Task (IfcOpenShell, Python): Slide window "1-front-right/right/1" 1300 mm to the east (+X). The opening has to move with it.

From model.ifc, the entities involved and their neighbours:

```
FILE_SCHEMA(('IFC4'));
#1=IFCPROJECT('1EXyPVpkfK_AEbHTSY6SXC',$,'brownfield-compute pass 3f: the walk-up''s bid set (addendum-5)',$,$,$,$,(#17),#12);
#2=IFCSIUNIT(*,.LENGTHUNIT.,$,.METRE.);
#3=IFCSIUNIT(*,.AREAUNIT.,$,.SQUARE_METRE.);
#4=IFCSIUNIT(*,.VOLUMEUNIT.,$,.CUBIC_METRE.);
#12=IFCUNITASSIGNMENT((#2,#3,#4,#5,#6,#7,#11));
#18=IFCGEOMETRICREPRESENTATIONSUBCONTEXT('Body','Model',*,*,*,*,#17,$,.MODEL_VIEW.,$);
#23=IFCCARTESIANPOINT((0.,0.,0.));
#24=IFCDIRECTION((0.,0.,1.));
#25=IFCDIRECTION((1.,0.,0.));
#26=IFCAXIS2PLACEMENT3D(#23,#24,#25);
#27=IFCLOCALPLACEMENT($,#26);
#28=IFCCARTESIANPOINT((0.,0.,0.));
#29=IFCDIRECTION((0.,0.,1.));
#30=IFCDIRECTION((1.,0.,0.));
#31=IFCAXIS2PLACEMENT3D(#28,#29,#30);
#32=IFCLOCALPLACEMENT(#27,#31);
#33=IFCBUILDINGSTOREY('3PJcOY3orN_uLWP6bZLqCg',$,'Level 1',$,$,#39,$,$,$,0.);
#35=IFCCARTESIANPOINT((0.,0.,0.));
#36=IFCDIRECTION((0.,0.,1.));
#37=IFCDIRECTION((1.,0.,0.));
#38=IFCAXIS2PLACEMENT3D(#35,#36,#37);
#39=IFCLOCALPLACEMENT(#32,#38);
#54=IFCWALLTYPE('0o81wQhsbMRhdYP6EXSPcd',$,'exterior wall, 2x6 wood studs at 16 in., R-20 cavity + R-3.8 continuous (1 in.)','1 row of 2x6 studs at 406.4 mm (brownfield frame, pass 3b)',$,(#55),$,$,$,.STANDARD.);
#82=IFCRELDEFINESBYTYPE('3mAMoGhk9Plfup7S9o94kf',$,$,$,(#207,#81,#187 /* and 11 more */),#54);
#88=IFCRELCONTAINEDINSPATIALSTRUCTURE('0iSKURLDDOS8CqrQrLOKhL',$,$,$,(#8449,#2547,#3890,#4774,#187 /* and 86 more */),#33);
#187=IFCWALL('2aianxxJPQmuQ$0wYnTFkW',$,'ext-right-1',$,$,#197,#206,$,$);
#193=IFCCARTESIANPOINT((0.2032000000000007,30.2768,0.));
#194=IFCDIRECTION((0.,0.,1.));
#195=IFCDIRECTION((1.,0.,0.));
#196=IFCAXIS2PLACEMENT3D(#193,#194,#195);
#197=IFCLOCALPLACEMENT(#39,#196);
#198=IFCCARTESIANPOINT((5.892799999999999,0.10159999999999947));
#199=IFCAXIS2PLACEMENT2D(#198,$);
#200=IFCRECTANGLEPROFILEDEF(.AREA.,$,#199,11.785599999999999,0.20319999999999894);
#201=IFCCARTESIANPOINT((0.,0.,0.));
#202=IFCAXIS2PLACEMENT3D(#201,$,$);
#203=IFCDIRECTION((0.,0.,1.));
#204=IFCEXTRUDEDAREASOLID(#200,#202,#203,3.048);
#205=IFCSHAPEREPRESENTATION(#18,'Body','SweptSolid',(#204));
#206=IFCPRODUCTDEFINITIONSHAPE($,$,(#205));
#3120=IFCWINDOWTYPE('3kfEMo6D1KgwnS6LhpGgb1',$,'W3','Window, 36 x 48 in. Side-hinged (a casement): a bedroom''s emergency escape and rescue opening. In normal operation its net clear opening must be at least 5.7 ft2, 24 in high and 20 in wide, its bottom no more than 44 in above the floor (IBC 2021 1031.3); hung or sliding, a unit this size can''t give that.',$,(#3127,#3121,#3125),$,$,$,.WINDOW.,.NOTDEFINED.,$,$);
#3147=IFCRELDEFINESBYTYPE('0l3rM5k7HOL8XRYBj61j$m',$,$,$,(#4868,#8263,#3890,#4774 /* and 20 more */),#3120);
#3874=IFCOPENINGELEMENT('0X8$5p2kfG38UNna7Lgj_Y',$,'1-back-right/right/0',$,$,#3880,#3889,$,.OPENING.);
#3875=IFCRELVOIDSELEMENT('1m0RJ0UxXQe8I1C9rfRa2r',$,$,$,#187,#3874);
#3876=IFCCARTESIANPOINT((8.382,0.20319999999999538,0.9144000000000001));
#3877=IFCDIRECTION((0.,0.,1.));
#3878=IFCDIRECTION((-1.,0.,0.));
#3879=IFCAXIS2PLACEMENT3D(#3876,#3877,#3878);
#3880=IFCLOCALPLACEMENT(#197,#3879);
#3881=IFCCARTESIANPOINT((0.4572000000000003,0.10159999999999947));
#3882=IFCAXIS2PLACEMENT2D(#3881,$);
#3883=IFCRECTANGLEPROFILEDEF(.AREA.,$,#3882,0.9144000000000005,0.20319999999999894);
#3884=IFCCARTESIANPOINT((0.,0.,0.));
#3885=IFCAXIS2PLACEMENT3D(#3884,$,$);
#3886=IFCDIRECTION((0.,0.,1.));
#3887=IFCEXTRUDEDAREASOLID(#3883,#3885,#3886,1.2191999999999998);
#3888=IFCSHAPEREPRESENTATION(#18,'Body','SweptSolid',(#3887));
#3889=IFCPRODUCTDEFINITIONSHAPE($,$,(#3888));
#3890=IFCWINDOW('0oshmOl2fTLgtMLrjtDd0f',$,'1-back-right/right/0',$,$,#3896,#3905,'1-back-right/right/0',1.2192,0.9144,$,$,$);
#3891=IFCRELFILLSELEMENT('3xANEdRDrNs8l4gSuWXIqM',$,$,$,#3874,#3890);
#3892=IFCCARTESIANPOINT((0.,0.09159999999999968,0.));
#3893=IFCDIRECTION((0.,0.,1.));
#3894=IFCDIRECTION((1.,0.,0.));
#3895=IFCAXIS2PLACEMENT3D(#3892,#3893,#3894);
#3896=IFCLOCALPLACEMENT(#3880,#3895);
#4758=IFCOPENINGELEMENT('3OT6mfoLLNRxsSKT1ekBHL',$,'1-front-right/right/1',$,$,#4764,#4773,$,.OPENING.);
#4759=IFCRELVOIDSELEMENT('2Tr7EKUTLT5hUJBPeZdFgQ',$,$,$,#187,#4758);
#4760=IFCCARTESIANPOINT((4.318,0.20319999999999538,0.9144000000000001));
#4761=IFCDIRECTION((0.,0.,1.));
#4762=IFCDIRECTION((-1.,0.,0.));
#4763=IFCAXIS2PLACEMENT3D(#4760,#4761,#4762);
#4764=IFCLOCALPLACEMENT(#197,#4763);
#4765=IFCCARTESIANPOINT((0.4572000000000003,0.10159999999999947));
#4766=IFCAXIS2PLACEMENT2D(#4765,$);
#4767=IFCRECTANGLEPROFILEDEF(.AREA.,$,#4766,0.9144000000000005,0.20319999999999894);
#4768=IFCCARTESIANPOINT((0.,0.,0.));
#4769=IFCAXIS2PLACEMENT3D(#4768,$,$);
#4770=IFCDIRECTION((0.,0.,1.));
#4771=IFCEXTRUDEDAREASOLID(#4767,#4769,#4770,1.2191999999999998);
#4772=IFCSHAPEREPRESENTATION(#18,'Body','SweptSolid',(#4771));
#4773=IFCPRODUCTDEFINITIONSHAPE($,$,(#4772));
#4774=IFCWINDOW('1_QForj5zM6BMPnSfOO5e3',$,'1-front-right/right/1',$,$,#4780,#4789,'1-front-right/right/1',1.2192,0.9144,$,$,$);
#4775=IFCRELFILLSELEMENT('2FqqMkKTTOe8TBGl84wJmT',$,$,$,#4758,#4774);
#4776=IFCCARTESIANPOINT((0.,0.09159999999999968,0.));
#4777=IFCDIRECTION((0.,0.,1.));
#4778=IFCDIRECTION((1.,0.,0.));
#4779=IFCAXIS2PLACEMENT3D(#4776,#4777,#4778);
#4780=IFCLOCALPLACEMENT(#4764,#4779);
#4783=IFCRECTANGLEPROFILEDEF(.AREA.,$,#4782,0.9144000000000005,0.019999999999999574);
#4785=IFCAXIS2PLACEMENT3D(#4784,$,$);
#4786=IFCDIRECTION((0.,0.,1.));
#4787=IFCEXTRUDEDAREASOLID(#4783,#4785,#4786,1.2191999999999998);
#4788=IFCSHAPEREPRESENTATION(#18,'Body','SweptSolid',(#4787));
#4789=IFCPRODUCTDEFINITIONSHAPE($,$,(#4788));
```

```python
import ifcopenshell
import ifcopenshell.api.geometry
import ifcopenshell.util.placement
import ifcopenshell.util.unit

model = ifcopenshell.open("model.ifc")
unit_scale = ifcopenshell.util.unit.calculate_unit_scale(model)

window = model.by_guid("1_QForj5zM6BMPnSfOO5e3")
opening = window.FillsVoids[0].RelatingOpeningElement
wall = opening.VoidsElements[0].RelatingBuildingElement

wall_matrix = ifcopenshell.util.placement.get_local_placement(wall.ObjectPlacement)
shift = wall_matrix[:3, 0] * 1.3 / unit_scale
before = ifcopenshell.util.placement.get_local_placement(window.ObjectPlacement)[:3, 3].copy()

# The window is placed relative to its opening, so it follows when the opening moves.
matrix = ifcopenshell.util.placement.get_local_placement(opening.ObjectPlacement)
matrix[:3, 3] += shift
ifcopenshell.api.geometry.edit_object_placement(
    model, product=opening, matrix=matrix, is_si=False, should_transform_children=True
)

after = ifcopenshell.util.placement.get_local_placement(window.ObjectPlacement)[:3, 3]
print("window moved by", (after - before).round(3) + 0.0)

model.write("model_rev.ifc")
```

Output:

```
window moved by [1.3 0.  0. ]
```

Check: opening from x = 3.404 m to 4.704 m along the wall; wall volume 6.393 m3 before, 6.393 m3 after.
